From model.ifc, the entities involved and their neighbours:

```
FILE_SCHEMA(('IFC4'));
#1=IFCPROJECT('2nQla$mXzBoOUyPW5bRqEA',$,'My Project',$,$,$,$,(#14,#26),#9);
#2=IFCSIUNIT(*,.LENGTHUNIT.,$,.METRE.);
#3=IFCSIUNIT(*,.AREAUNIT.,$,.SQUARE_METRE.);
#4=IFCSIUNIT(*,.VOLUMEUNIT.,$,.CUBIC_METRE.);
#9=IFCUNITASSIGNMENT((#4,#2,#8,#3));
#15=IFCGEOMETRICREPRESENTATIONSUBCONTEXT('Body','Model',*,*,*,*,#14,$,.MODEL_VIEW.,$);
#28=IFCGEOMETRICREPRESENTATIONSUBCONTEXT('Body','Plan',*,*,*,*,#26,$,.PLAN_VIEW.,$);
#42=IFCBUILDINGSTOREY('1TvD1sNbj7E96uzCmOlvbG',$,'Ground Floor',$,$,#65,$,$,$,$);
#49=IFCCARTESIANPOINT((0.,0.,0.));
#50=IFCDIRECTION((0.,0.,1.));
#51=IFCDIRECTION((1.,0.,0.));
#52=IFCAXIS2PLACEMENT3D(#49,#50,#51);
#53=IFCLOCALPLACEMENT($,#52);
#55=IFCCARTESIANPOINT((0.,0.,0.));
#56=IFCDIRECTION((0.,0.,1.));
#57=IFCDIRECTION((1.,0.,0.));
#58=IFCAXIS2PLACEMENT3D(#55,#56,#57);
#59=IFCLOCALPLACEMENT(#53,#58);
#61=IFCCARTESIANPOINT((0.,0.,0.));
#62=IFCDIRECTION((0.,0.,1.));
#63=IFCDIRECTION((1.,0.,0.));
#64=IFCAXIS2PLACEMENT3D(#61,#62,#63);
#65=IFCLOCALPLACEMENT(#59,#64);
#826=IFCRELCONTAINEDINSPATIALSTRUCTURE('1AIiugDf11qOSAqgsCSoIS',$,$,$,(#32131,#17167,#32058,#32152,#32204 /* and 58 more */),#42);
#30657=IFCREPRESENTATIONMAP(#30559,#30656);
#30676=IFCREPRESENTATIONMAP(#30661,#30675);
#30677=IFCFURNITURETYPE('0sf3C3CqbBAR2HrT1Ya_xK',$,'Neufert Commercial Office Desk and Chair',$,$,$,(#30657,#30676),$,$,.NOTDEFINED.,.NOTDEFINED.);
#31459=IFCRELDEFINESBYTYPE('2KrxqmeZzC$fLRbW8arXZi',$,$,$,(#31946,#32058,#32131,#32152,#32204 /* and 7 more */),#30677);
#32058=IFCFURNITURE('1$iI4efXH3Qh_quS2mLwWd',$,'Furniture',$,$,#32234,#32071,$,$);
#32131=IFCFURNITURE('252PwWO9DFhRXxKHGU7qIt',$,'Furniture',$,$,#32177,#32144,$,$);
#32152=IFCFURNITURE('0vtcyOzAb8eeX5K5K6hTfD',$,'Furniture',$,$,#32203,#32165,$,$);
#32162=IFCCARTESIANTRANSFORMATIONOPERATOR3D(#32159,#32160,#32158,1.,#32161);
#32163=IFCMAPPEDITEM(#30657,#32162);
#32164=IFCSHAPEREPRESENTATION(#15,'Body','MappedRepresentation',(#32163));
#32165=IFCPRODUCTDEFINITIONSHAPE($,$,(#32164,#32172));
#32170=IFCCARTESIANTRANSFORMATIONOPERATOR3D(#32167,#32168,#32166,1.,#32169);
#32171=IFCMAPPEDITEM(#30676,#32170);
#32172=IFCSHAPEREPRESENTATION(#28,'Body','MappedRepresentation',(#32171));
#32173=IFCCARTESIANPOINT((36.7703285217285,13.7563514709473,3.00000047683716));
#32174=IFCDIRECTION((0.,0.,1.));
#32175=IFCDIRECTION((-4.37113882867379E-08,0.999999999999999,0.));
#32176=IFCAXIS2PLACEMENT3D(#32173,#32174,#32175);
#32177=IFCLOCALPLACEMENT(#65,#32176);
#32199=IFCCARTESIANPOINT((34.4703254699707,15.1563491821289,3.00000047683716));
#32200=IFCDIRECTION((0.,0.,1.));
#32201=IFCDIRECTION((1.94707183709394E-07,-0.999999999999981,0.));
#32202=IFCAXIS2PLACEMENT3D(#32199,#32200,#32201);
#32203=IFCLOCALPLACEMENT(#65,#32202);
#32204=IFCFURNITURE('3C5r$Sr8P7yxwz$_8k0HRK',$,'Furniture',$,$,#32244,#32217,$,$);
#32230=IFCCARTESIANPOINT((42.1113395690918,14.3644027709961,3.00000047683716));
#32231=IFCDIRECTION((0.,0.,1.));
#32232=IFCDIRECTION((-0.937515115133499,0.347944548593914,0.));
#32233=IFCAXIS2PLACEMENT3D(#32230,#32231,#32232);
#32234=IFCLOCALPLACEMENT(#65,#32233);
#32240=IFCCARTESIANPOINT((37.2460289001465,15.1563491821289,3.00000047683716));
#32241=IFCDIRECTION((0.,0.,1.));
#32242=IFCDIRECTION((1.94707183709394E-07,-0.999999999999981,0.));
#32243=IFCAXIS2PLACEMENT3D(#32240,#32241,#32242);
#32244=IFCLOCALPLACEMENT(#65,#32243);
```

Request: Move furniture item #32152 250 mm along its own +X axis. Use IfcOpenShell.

```python
import ifcopenshell
import ifcopenshell.api.geometry
import ifcopenshell.util.placement
import ifcopenshell.util.unit

model = ifcopenshell.open("model.ifc")
unit_scale = ifcopenshell.util.unit.calculate_unit_scale(model)

item = model.by_guid("0vtcyOzAb8eeX5K5K6hTfD")
matrix = ifcopenshell.util.placement.get_local_placement(item.ObjectPlacement)
matrix[:3, 3] += matrix[:3, 0] * 0.25 / unit_scale
ifcopenshell.api.geometry.edit_object_placement(model, product=item, matrix=matrix, is_si=False)

print(ifcopenshell.util.placement.get_local_placement(item.ObjectPlacement).round(3) + 0.0)

model.write("model_edited.ifc")
```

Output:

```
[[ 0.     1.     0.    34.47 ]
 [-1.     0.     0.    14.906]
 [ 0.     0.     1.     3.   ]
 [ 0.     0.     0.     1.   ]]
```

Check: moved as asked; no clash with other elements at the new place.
